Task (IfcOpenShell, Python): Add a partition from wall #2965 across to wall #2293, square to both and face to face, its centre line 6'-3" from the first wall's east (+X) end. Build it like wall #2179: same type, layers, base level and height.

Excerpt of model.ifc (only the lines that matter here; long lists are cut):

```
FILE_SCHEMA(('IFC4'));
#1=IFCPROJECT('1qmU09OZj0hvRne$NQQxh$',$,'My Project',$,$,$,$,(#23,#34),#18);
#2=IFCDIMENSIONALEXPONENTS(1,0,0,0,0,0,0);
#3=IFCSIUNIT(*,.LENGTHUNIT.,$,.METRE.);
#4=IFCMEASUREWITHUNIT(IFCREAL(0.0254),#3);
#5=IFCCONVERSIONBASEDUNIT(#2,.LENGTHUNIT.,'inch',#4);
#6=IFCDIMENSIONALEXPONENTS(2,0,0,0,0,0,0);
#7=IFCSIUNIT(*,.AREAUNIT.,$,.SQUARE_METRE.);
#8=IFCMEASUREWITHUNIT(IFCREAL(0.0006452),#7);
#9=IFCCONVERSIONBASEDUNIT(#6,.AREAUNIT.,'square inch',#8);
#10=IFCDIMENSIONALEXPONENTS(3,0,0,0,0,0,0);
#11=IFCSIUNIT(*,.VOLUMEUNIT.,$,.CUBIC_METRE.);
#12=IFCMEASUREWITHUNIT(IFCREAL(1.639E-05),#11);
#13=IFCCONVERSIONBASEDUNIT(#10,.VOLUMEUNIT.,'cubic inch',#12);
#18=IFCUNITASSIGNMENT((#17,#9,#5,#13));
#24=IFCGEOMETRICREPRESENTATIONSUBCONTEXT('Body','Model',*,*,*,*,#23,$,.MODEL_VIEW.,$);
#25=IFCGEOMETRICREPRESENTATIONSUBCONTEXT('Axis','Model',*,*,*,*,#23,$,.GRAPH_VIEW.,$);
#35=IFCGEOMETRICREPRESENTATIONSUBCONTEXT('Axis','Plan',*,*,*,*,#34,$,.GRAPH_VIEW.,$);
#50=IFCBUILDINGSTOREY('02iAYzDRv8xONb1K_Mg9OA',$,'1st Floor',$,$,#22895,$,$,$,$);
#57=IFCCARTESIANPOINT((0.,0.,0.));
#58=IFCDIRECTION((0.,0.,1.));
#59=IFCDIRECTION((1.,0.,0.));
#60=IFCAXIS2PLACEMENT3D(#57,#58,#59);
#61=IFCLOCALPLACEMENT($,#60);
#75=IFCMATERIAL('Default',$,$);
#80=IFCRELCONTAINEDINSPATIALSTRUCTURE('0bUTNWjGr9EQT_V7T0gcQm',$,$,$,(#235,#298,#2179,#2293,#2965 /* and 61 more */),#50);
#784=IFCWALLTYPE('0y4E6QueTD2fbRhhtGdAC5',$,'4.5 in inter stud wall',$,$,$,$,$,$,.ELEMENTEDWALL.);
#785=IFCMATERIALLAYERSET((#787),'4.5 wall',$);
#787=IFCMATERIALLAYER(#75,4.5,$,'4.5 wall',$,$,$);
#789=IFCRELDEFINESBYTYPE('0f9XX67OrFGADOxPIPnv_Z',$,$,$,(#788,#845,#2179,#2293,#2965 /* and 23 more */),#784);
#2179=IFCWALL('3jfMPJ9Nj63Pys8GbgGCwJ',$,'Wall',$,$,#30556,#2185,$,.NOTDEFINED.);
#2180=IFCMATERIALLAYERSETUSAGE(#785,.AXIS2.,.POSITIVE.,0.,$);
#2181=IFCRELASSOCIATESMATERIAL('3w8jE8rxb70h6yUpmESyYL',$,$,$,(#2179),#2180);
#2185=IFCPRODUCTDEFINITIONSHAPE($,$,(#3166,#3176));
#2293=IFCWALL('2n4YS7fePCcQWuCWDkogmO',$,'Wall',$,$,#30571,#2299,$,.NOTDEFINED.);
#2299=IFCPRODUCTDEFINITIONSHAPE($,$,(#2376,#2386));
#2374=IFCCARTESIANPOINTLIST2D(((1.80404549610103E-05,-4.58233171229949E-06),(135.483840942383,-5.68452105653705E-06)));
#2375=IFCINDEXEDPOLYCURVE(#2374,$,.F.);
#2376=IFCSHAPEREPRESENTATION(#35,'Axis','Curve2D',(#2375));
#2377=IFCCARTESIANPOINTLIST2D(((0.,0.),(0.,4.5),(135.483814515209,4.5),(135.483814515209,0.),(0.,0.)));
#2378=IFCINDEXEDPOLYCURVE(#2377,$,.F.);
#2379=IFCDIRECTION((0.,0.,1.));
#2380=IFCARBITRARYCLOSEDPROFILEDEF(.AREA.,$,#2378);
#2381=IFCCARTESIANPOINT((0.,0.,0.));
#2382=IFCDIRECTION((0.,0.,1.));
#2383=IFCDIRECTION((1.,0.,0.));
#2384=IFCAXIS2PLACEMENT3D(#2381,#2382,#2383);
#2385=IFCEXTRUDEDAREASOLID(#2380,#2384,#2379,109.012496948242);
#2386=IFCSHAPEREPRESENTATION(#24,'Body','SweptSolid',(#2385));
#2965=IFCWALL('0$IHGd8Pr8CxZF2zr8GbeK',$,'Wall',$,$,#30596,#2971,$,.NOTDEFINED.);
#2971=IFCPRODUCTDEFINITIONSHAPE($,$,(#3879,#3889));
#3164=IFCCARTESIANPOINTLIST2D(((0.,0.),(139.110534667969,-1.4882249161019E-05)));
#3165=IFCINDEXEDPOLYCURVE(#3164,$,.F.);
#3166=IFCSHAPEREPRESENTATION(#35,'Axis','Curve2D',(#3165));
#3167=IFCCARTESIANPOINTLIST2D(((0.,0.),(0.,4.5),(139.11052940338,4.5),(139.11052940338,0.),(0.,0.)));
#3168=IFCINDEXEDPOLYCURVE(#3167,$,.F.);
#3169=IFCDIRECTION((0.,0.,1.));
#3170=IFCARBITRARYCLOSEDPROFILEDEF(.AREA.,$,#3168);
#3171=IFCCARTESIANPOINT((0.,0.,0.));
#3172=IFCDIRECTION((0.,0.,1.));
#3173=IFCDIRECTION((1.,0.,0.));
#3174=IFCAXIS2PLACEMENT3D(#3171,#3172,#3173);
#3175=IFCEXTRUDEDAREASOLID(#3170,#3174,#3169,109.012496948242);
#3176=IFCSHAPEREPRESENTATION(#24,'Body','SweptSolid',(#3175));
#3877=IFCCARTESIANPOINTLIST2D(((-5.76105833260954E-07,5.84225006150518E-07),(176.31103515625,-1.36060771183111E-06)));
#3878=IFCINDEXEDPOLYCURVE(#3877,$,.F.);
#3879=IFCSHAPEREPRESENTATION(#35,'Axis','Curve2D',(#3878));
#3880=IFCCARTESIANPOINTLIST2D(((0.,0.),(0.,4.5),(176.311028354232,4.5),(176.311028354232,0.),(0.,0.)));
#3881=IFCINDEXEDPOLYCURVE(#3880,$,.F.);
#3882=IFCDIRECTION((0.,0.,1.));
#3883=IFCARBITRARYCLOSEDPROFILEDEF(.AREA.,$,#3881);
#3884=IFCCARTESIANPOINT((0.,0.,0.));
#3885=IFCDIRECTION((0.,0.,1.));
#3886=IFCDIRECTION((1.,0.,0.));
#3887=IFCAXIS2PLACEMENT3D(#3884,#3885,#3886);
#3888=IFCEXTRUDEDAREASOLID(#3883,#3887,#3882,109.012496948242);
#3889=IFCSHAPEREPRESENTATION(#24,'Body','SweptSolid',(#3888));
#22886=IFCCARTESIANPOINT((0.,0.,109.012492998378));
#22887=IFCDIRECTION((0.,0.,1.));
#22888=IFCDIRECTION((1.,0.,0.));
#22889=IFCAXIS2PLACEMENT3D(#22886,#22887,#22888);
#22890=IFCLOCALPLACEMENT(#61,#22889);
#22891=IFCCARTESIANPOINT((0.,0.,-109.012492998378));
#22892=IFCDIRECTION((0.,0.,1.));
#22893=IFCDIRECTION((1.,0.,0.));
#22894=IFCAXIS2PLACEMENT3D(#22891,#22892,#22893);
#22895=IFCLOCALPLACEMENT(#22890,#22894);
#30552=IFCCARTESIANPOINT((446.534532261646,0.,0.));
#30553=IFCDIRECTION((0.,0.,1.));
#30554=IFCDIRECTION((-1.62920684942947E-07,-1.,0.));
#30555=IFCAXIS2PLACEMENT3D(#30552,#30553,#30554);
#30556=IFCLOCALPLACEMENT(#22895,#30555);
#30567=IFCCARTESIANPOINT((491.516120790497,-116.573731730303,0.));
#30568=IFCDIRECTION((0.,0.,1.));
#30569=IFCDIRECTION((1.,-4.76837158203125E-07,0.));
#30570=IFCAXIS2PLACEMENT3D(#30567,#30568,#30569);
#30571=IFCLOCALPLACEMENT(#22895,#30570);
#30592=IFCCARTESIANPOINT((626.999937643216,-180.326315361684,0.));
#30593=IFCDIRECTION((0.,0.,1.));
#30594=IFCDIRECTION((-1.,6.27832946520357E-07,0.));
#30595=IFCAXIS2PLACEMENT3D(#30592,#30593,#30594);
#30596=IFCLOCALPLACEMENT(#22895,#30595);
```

```python
import numpy as np
import ifcopenshell
import ifcopenshell.api.geometry
import ifcopenshell.api.material
import ifcopenshell.api.pset
import ifcopenshell.api.root
import ifcopenshell.api.spatial
import ifcopenshell.api.type
import ifcopenshell.geom
import ifcopenshell.util.element
import ifcopenshell.util.placement
import ifcopenshell.util.representation
import ifcopenshell.util.shape
import ifcopenshell.util.unit

model = ifcopenshell.open("model.ifc")
unit_scale = ifcopenshell.util.unit.calculate_unit_scale(model)
settings = ifcopenshell.geom.settings()
settings.set("use-world-coords", True)

start_wall = model.by_guid("0$IHGd8Pr8CxZF2zr8GbeK")
end_wall = model.by_id(2293)
like = model.by_guid("3jfMPJ9Nj63Pys8GbgGCwJ")
matrix = ifcopenshell.util.placement.get_local_placement(start_wall.ObjectPlacement)
matrix[:3, 3] *= unit_scale


def extent(element):
    """Bounding box in the first wall's axes, in metres."""
    shape = ifcopenshell.geom.create_shape(settings, element)
    points = (ifcopenshell.util.shape.get_vertices(shape.geometry) - matrix[:3, 3]) @ matrix[:3, :3]
    return points.min(axis=0), points.max(axis=0)


y_start = extent(start_wall)[0][1]
y_end = extent(end_wall)[1][1]
like_min, like_max = extent(like)
length, height = float(abs(y_end - y_start)), float(like_max[2] - like_min[2])
layer_set = ifcopenshell.util.element.get_material(like, should_skip_usage=True)
thickness = sum(layer.LayerThickness for layer in layer_set.MaterialLayers) * unit_scale

wall = ifcopenshell.api.root.create_entity(model, ifc_class="IfcWall", name="New partition")
storey = ifcopenshell.util.element.get_container(like)
ifcopenshell.api.spatial.assign_container(model, products=[wall], relating_structure=storey)
ifcopenshell.api.type.assign_type(
    model, related_objects=[wall], relating_type=ifcopenshell.util.element.get_type(like), should_map_representations=False
)
rel = ifcopenshell.api.material.assign_material(
    model, products=[wall], type="IfcMaterialLayerSetUsage", material=layer_set
)
rel.RelatingMaterial.OffsetFromReferenceLine = -thickness / 2 / unit_scale
pset = ifcopenshell.api.pset.add_pset(model, product=wall, name="Pset_WallCommon")
ifcopenshell.api.pset.edit_pset(model, pset=pset, properties={"IsExternal": False, "LoadBearing": False})

# The axis runs down the middle of the wall.
axis = ifcopenshell.api.geometry.add_axis_representation(
    model, context=ifcopenshell.util.representation.get_context(model, "Model", "Axis"), axis=[(0.0, 0.0), (length, 0.0)]
)
body = ifcopenshell.api.geometry.add_wall_representation(
    model,
    context=ifcopenshell.util.representation.get_context(model, "Model", "Body", "MODEL_VIEW"),
    length=length,
    height=height,
    thickness=thickness,
    offset=-thickness / 2,
)
for representation in (axis, body):
    ifcopenshell.api.geometry.assign_representation(model, product=wall, representation=representation)

placement = matrix @ ifcopenshell.util.placement.rotation(-90, "Z")
placement[:, 3] = matrix @ np.array([extent(start_wall)[0][0] + 1.905, y_start, like_min[2], 1.0])
ifcopenshell.api.geometry.edit_object_placement(model, product=wall, matrix=placement)

print(f"partition {length:.3f} m long, {height:.3f} m high, {thickness:.3f} m thick")

model.write("model_rev.ifc")
```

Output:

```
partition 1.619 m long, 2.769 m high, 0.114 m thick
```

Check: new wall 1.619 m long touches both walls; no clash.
